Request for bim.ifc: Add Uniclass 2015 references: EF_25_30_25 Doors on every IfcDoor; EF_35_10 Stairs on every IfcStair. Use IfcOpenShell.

First a look at what the model holds.

```python
import ifcopenshell

model = ifcopenshell.open("bim.ifc")
print(model.schema)
print("classifications:", [c.Name for c in model.by_type("IfcClassification")])
for ifc_class in ("IfcDoor", "IfcRoof", "IfcStair", "IfcWall", "IfcWindow"):
    print(ifc_class, len(model.by_type(ifc_class)))
```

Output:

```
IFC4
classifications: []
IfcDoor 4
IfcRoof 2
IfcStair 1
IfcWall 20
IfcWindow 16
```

```python
import ifcopenshell
import ifcopenshell.api.classification

model = ifcopenshell.open("bim.ifc")

system = ifcopenshell.api.classification.add_classification(model, classification="Uniclass 2015")

codes = {
    "IfcDoor": ("EF_25_30_25", "Doors"),
    "IfcStair": ("EF_35_10", "Stairs"),
}
for ifc_class, (code, name) in codes.items():
    products = model.by_type(ifc_class)
    ifcopenshell.api.classification.add_reference(
        model, products=products, classification=system, identification=code, name=name
    )
    print(code, len(products))

model.write("bim_rev.ifc")
```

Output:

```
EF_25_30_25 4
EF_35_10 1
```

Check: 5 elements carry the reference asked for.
